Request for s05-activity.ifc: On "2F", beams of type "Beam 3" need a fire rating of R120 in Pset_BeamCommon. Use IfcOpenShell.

First a look at what the model holds.

```python
import ifcopenshell
import ifcopenshell.util.element

model = ifcopenshell.open("s05-activity.ifc")
print(model.schema)
storey = next(s for s in model.by_type("IfcBuildingStorey") if s.Name == "2F")
beams = [e for e in ifcopenshell.util.element.get_decomposition(storey) if e.is_a("IfcBeam")]
seen = {}
for e in beams:
    element_type = ifcopenshell.util.element.get_type(e)
    key = (element_type.Name if element_type != e and element_type else None, ifcopenshell.util.element.get_pset(e, "Pset_BeamCommon", "FireRating"))
    seen[key] = seen.get(key, 0) + 1
for (name, value), count in sorted(seen.items(), key=str):
    print(count, "x", name, "|", value)
```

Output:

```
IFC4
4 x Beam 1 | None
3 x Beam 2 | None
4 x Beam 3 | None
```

```python
import ifcopenshell
import ifcopenshell.api.pset
import ifcopenshell.util.element

model = ifcopenshell.open("s05-activity.ifc")

storey = next(s for s in model.by_type("IfcBuildingStorey") if s.Name == "2F")
beams = [e for e in ifcopenshell.util.element.get_decomposition(storey) if e.is_a("IfcBeam")]

count = 0
for e in beams:
    element_type = ifcopenshell.util.element.get_type(e)
    if element_type in (None, e) or element_type.Name != "Beam 3":
        continue
    # add_pset returns the element's existing set when there is one.
    pset = ifcopenshell.api.pset.add_pset(model, product=e, name="Pset_BeamCommon")
    ifcopenshell.api.pset.edit_pset(model, pset=pset, properties={"FireRating": "R120"})
    count += 1

print(count, "beams updated")

model.write("s05-activity-out.ifc")
```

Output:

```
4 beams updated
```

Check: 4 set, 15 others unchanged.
